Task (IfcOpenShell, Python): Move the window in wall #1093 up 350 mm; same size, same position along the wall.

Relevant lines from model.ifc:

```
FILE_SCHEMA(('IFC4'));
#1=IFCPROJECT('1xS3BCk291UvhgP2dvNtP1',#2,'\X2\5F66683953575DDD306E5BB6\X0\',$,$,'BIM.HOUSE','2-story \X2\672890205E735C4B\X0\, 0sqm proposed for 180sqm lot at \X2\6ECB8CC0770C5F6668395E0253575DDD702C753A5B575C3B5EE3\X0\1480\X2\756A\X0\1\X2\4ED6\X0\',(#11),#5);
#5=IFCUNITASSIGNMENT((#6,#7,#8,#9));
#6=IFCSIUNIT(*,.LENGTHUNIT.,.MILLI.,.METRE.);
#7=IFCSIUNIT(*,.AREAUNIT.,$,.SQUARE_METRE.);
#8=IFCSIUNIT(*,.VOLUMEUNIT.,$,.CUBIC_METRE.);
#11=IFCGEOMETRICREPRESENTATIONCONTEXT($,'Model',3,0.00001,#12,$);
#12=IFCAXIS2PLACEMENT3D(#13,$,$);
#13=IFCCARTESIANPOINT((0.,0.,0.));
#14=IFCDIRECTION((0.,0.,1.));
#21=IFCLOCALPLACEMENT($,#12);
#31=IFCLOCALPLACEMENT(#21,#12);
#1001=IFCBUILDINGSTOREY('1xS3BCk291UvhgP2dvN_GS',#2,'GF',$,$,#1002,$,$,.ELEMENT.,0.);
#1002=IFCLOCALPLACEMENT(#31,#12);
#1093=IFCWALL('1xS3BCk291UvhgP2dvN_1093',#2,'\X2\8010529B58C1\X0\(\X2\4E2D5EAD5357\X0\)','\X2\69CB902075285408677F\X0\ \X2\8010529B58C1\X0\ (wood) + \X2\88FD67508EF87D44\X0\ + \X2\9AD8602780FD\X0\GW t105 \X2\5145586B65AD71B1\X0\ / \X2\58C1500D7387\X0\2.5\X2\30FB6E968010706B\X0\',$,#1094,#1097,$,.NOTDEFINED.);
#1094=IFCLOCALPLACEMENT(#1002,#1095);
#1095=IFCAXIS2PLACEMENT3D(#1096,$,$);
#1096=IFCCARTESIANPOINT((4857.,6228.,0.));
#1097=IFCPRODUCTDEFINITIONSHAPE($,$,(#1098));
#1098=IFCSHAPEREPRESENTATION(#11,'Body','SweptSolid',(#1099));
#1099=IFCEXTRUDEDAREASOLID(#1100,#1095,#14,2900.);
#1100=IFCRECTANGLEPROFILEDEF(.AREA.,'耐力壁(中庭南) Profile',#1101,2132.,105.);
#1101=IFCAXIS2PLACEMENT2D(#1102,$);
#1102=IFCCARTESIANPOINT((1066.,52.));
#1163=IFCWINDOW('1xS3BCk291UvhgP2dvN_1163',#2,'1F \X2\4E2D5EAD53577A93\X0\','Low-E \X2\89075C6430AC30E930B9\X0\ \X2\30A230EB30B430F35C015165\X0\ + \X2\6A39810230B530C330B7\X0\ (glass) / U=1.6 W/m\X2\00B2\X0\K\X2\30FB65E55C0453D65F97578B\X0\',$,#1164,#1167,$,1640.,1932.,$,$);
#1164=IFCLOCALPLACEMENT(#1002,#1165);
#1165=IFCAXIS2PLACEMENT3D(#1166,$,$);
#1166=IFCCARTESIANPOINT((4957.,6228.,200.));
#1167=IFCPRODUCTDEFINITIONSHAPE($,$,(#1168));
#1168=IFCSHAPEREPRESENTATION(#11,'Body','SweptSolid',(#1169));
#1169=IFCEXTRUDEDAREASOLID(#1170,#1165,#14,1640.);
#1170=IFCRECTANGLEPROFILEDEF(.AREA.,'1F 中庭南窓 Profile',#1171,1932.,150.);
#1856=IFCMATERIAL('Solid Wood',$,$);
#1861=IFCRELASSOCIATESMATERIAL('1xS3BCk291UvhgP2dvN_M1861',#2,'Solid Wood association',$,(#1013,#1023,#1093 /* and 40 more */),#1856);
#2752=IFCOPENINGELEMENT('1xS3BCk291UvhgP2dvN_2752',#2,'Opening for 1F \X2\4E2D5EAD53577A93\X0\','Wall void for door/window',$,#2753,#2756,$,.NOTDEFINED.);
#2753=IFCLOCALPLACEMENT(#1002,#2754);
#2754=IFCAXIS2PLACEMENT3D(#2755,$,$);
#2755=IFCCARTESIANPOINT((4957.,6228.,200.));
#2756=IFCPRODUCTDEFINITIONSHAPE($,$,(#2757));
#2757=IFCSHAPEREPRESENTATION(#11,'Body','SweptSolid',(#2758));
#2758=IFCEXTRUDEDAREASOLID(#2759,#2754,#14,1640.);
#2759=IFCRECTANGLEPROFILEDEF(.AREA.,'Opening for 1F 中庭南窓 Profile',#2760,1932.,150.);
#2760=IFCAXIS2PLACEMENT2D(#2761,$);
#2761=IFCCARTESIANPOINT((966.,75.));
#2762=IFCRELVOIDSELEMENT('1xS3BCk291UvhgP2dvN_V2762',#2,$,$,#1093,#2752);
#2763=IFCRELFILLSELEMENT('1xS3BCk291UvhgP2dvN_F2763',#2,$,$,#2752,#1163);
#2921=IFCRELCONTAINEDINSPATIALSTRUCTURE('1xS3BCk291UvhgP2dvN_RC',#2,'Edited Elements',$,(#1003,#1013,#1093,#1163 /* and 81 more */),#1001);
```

```python
import numpy as np
import ifcopenshell
import ifcopenshell.api.geometry
import ifcopenshell.util.placement
import ifcopenshell.util.unit

model = ifcopenshell.open("model.ifc")
unit_scale = ifcopenshell.util.unit.calculate_unit_scale(model)

window = model.by_guid("1xS3BCk291UvhgP2dvN_1163")
opening = window.FillsVoids[0].RelatingOpeningElement
dz = 350.0

shift = np.array([0.0, 0.0, dz])
# The window is not placed relative to its opening, so move both.
for product in (opening, window):
    matrix = ifcopenshell.util.placement.get_local_placement(product.ObjectPlacement)
    matrix[:3, 3] += shift
    ifcopenshell.api.geometry.edit_object_placement(model, product=product, matrix=matrix, is_si=False)

print(f"moved by {dz * unit_scale:+.3f} m")

model.write("model_updated.ifc")
```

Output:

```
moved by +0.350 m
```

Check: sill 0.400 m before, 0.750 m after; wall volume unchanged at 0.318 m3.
